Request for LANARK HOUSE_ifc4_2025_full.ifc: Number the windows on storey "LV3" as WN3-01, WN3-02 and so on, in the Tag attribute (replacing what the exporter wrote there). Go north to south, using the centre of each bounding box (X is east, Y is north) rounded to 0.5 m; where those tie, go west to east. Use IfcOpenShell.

First a look at what the model holds.

```python
import ifcopenshell
import ifcopenshell.util.element
import ifcopenshell.util.placement

model = ifcopenshell.open("LANARK HOUSE_ifc4_2025_full.ifc")
print(model.schema)
storey = next(s for s in model.by_type("IfcBuildingStorey") if s.Name == "LV3")
windows = [e for e in ifcopenshell.util.element.get_decomposition(storey) if e.is_a("IfcWindow")]
for e in sorted(windows, key=lambda e: e.id()):
    origin = ifcopenshell.util.placement.get_local_placement(e.ObjectPlacement)[:3, 3]
    print(e.id(), e.Tag, e.Name, origin.round(2) + 0.0, sep=" | ")
```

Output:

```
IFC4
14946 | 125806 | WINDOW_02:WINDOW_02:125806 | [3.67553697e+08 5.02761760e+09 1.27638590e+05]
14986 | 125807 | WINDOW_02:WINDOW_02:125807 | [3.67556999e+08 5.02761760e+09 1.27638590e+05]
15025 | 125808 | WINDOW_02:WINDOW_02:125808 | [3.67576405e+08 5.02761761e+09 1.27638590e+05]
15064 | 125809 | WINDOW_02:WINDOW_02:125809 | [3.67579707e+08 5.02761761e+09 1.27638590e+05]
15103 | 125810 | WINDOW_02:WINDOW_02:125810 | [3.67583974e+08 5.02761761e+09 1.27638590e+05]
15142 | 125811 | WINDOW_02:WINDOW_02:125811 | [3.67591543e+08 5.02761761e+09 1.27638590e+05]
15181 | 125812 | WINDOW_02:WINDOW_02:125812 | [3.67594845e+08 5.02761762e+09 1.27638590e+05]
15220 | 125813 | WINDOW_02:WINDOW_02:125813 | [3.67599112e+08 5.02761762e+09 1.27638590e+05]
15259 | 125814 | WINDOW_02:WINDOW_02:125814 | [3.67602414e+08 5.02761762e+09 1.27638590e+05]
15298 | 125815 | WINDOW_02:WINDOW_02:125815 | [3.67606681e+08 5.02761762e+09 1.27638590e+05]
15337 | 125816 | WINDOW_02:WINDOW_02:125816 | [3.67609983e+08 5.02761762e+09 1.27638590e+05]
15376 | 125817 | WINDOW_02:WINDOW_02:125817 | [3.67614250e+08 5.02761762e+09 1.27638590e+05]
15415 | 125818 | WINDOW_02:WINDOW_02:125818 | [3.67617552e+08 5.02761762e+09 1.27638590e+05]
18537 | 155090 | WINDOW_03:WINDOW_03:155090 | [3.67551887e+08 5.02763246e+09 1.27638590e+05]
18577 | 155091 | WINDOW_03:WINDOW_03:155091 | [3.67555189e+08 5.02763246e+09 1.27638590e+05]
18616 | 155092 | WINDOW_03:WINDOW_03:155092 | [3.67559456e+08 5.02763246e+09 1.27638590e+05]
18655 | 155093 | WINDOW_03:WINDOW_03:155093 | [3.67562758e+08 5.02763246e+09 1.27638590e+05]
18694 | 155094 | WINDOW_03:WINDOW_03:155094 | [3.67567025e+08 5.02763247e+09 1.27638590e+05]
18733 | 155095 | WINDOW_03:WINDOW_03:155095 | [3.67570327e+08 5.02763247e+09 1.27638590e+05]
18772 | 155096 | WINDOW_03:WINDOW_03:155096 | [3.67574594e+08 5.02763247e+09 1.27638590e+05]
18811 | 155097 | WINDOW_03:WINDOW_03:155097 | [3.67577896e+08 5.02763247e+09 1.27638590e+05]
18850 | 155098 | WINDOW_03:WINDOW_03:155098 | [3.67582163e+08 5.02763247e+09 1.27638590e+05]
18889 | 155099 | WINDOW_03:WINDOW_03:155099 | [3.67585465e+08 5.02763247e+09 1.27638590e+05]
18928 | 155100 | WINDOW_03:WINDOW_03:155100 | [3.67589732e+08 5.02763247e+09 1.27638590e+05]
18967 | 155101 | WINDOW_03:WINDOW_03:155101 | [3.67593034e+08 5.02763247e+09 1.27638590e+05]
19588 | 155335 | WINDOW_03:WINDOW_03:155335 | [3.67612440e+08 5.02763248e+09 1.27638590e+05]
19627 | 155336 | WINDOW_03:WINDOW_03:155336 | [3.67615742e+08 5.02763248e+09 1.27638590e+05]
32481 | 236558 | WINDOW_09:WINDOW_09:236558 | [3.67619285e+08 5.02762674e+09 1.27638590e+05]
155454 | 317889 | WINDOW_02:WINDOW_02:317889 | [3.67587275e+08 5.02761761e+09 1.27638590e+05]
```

```python
import ifcopenshell
import ifcopenshell.geom
import ifcopenshell.util.element
import ifcopenshell.util.shape

model = ifcopenshell.open("LANARK HOUSE_ifc4_2025_full.ifc")
settings = ifcopenshell.geom.settings()
settings.set("use-world-coords", True)


def centre(element):
    shape = ifcopenshell.geom.create_shape(settings, element)
    return ifcopenshell.util.shape.get_bbox_centroid(shape.geometry)


storey = next(s for s in model.by_type("IfcBuildingStorey") if s.Name == "LV3")
windows = [e for e in ifcopenshell.util.element.get_decomposition(storey) if e.is_a("IfcWindow")]

# Insertion points can sit at a corner or the storey origin, so sort by the geometry (in metres).
centres = {e: centre(e) for e in windows}
windows.sort(key=lambda e: (-round(centres[e][1] / 0.5), centres[e][0]))

for i, e in enumerate(windows, start=1):
    number = f"WN3-{i:02d}"
    e.Tag = number
    print(e.id(), number)

model.write("LANARK HOUSE_ifc4_2025_full_edited.ifc")
```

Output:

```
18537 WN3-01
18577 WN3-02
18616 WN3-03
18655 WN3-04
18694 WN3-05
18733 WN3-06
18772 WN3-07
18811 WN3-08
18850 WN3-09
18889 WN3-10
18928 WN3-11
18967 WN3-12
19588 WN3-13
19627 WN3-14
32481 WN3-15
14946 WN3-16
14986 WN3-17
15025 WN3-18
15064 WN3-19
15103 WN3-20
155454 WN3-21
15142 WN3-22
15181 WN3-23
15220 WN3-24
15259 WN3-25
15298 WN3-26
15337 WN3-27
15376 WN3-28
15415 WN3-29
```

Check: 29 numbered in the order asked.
